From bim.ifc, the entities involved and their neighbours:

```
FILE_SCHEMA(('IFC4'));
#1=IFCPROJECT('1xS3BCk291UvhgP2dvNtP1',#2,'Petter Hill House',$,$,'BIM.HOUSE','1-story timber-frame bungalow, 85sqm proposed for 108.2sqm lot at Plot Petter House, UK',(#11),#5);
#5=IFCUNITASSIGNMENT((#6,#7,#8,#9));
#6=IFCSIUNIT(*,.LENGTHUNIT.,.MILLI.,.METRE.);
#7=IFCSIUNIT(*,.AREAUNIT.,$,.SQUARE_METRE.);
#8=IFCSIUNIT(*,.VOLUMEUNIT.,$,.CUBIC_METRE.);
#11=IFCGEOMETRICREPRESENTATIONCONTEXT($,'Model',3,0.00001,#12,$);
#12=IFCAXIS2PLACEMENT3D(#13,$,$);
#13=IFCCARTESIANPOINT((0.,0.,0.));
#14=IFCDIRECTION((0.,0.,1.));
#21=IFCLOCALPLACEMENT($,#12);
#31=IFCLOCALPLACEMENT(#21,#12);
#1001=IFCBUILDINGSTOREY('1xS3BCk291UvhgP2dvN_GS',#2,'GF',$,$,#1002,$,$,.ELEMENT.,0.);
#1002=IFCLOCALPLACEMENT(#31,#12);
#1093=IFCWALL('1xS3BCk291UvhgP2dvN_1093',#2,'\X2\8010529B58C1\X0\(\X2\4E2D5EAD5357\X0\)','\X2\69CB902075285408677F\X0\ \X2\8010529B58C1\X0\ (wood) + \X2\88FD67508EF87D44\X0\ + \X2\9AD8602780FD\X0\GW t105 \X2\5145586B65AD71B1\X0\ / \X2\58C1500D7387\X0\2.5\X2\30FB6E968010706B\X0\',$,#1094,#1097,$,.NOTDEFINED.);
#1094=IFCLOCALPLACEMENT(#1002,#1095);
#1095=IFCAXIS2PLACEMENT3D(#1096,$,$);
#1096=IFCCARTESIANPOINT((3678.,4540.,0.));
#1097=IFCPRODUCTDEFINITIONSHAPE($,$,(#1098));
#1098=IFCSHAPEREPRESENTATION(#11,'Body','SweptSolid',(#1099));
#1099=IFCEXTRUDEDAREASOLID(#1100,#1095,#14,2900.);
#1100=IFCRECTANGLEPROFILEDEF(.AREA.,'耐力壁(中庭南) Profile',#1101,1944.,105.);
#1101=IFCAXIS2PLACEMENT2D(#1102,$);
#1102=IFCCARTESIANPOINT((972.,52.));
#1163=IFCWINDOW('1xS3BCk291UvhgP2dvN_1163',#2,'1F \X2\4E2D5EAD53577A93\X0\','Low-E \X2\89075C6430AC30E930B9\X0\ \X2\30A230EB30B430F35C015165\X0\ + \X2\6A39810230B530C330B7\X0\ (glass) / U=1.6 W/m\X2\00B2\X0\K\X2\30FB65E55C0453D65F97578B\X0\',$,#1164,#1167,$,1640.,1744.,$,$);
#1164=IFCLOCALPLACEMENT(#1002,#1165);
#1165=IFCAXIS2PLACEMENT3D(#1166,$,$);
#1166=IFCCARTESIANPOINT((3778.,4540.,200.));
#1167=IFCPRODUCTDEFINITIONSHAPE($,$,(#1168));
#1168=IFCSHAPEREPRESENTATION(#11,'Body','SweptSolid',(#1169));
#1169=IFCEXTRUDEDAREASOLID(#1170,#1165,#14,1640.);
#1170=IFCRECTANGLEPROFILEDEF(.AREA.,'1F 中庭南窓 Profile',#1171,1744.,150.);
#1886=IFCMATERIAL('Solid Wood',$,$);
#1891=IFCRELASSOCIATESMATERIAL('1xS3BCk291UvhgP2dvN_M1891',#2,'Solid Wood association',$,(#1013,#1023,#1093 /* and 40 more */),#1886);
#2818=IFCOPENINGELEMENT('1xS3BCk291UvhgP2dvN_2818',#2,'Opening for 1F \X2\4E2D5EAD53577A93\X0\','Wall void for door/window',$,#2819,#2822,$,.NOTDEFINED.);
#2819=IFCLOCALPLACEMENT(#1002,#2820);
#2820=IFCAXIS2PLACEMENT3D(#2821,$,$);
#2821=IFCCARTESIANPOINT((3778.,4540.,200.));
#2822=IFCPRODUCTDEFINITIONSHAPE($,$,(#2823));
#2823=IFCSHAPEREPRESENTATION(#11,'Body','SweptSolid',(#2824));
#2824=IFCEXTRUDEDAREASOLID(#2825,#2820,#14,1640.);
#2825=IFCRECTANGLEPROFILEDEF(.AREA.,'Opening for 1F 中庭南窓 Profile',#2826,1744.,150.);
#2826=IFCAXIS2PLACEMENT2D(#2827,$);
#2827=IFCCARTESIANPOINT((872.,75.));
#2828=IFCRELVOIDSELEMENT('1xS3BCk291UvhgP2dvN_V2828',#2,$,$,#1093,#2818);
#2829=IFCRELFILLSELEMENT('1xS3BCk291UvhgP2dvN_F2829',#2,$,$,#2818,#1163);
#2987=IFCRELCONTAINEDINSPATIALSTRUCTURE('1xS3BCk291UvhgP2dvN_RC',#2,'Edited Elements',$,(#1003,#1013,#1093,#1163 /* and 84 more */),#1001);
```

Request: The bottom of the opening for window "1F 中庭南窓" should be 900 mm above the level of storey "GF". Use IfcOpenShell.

```python
import numpy as np
import ifcopenshell
import ifcopenshell.api.geometry
import ifcopenshell.geom
import ifcopenshell.util.element
import ifcopenshell.util.placement
import ifcopenshell.util.shape
import ifcopenshell.util.unit

model = ifcopenshell.open("bim.ifc")
unit_scale = ifcopenshell.util.unit.calculate_unit_scale(model)

window = model.by_guid("1xS3BCk291UvhgP2dvN_1163")
opening = window.FillsVoids[0].RelatingOpeningElement
storey = ifcopenshell.util.element.get_container(window, ifc_class="IfcBuildingStorey")
level = ifcopenshell.util.placement.get_local_placement(storey.ObjectPlacement)[2, 3]

# The opening's origin need not be at the sill, so measure its lowest point.
shape = ifcopenshell.geom.create_shape(ifcopenshell.geom.settings(), opening)
bottom = ifcopenshell.util.shape.get_shape_bottom_elevation(shape, shape.geometry) / unit_scale
dz = level + 0.9 / unit_scale - bottom

shift = np.array([0.0, 0.0, dz])
# The window is not placed relative to its opening, so move both.
for product in (opening, window):
    matrix = ifcopenshell.util.placement.get_local_placement(product.ObjectPlacement)
    matrix[:3, 3] += shift
    ifcopenshell.api.geometry.edit_object_placement(model, product=product, matrix=matrix, is_si=False)

print(f"moved by {dz * unit_scale:+.3f} m")

model.write("bim_edited.ifc")
```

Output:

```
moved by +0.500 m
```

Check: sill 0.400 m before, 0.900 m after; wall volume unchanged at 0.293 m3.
